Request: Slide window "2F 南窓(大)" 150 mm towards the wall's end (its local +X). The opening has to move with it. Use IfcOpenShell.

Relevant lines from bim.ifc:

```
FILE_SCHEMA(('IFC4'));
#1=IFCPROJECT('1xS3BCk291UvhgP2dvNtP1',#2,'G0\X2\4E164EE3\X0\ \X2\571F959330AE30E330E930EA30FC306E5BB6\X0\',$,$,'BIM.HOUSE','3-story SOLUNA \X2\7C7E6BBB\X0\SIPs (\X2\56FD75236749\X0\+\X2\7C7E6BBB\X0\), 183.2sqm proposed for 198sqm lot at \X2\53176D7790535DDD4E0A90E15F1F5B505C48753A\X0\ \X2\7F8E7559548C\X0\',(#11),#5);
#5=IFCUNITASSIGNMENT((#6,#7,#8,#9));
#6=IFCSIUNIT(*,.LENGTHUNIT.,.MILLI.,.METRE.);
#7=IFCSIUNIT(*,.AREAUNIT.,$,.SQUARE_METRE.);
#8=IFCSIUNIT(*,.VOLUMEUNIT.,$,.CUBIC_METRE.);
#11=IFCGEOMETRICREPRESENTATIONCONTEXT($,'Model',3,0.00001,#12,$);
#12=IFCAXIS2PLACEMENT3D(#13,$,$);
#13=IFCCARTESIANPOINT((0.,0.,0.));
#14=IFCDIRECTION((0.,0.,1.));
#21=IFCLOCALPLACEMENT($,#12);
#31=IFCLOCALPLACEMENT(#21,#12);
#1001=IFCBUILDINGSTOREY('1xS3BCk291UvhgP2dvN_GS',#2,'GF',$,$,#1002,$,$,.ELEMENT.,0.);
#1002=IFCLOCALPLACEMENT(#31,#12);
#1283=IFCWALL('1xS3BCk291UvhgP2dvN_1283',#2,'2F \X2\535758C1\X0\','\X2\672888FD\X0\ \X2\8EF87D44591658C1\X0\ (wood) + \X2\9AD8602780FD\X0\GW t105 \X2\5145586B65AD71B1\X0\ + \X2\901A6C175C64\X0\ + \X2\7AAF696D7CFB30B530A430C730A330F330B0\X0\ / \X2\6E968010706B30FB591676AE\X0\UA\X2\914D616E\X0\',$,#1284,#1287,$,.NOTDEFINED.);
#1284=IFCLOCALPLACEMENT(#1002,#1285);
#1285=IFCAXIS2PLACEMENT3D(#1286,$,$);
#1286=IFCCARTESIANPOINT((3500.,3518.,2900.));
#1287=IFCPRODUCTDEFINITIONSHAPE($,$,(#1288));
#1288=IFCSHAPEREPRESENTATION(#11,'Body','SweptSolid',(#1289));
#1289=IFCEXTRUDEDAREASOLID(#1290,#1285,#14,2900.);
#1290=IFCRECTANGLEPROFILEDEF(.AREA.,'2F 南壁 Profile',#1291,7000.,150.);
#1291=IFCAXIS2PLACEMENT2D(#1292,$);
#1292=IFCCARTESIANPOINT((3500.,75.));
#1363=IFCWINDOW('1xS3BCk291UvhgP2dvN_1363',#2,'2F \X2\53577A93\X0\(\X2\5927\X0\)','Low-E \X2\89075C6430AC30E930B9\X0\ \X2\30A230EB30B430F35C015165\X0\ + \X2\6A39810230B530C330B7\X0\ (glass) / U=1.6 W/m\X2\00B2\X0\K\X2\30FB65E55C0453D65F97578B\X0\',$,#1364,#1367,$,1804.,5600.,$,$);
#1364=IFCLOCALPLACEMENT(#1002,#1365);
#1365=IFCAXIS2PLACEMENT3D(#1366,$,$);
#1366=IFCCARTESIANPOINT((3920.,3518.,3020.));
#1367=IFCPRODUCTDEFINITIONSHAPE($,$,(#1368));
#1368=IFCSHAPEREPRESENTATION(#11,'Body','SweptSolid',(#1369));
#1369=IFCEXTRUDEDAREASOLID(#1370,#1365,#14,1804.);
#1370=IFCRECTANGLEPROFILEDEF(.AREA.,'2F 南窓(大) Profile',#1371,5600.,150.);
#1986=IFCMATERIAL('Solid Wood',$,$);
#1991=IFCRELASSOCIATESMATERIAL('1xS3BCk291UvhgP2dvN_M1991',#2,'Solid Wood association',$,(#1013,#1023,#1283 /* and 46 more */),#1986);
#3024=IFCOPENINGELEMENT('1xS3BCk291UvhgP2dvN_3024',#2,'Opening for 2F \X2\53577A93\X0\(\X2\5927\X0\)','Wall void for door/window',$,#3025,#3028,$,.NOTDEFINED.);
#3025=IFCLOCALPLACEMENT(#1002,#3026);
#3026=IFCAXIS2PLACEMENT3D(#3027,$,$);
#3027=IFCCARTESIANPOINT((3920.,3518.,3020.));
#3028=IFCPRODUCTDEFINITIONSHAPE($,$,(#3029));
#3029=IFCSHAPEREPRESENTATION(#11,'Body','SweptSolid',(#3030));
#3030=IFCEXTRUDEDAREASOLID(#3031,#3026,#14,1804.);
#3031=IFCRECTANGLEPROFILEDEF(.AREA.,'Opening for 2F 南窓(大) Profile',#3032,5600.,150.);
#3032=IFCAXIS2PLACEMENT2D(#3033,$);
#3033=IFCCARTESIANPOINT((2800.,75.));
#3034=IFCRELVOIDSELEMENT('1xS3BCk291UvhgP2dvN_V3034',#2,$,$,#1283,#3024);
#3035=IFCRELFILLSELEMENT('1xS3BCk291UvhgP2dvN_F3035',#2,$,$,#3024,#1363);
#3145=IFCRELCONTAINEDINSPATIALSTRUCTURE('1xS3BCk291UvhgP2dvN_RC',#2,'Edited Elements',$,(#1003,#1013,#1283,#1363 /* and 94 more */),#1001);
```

```python
import ifcopenshell
import ifcopenshell.api.geometry
import ifcopenshell.util.placement
import ifcopenshell.util.unit

model = ifcopenshell.open("bim.ifc")
unit_scale = ifcopenshell.util.unit.calculate_unit_scale(model)

window = model.by_guid("1xS3BCk291UvhgP2dvN_1363")
opening = window.FillsVoids[0].RelatingOpeningElement
wall = opening.VoidsElements[0].RelatingBuildingElement

wall_matrix = ifcopenshell.util.placement.get_local_placement(wall.ObjectPlacement)
shift = wall_matrix[:3, 0] * 0.15 / unit_scale
before = ifcopenshell.util.placement.get_local_placement(window.ObjectPlacement)[:3, 3].copy()

# The window is not placed relative to its opening, so move both.
for product in (opening, window):
    matrix = ifcopenshell.util.placement.get_local_placement(product.ObjectPlacement)
    matrix[:3, 3] += shift
    ifcopenshell.api.geometry.edit_object_placement(model, product=product, matrix=matrix, is_si=False)

after = ifcopenshell.util.placement.get_local_placement(window.ObjectPlacement)[:3, 3]
print("window moved by", (after - before).round(3) + 0.0)

model.write("bim_edited.ifc")
```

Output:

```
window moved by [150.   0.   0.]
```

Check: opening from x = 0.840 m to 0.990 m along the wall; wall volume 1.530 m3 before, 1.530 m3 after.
